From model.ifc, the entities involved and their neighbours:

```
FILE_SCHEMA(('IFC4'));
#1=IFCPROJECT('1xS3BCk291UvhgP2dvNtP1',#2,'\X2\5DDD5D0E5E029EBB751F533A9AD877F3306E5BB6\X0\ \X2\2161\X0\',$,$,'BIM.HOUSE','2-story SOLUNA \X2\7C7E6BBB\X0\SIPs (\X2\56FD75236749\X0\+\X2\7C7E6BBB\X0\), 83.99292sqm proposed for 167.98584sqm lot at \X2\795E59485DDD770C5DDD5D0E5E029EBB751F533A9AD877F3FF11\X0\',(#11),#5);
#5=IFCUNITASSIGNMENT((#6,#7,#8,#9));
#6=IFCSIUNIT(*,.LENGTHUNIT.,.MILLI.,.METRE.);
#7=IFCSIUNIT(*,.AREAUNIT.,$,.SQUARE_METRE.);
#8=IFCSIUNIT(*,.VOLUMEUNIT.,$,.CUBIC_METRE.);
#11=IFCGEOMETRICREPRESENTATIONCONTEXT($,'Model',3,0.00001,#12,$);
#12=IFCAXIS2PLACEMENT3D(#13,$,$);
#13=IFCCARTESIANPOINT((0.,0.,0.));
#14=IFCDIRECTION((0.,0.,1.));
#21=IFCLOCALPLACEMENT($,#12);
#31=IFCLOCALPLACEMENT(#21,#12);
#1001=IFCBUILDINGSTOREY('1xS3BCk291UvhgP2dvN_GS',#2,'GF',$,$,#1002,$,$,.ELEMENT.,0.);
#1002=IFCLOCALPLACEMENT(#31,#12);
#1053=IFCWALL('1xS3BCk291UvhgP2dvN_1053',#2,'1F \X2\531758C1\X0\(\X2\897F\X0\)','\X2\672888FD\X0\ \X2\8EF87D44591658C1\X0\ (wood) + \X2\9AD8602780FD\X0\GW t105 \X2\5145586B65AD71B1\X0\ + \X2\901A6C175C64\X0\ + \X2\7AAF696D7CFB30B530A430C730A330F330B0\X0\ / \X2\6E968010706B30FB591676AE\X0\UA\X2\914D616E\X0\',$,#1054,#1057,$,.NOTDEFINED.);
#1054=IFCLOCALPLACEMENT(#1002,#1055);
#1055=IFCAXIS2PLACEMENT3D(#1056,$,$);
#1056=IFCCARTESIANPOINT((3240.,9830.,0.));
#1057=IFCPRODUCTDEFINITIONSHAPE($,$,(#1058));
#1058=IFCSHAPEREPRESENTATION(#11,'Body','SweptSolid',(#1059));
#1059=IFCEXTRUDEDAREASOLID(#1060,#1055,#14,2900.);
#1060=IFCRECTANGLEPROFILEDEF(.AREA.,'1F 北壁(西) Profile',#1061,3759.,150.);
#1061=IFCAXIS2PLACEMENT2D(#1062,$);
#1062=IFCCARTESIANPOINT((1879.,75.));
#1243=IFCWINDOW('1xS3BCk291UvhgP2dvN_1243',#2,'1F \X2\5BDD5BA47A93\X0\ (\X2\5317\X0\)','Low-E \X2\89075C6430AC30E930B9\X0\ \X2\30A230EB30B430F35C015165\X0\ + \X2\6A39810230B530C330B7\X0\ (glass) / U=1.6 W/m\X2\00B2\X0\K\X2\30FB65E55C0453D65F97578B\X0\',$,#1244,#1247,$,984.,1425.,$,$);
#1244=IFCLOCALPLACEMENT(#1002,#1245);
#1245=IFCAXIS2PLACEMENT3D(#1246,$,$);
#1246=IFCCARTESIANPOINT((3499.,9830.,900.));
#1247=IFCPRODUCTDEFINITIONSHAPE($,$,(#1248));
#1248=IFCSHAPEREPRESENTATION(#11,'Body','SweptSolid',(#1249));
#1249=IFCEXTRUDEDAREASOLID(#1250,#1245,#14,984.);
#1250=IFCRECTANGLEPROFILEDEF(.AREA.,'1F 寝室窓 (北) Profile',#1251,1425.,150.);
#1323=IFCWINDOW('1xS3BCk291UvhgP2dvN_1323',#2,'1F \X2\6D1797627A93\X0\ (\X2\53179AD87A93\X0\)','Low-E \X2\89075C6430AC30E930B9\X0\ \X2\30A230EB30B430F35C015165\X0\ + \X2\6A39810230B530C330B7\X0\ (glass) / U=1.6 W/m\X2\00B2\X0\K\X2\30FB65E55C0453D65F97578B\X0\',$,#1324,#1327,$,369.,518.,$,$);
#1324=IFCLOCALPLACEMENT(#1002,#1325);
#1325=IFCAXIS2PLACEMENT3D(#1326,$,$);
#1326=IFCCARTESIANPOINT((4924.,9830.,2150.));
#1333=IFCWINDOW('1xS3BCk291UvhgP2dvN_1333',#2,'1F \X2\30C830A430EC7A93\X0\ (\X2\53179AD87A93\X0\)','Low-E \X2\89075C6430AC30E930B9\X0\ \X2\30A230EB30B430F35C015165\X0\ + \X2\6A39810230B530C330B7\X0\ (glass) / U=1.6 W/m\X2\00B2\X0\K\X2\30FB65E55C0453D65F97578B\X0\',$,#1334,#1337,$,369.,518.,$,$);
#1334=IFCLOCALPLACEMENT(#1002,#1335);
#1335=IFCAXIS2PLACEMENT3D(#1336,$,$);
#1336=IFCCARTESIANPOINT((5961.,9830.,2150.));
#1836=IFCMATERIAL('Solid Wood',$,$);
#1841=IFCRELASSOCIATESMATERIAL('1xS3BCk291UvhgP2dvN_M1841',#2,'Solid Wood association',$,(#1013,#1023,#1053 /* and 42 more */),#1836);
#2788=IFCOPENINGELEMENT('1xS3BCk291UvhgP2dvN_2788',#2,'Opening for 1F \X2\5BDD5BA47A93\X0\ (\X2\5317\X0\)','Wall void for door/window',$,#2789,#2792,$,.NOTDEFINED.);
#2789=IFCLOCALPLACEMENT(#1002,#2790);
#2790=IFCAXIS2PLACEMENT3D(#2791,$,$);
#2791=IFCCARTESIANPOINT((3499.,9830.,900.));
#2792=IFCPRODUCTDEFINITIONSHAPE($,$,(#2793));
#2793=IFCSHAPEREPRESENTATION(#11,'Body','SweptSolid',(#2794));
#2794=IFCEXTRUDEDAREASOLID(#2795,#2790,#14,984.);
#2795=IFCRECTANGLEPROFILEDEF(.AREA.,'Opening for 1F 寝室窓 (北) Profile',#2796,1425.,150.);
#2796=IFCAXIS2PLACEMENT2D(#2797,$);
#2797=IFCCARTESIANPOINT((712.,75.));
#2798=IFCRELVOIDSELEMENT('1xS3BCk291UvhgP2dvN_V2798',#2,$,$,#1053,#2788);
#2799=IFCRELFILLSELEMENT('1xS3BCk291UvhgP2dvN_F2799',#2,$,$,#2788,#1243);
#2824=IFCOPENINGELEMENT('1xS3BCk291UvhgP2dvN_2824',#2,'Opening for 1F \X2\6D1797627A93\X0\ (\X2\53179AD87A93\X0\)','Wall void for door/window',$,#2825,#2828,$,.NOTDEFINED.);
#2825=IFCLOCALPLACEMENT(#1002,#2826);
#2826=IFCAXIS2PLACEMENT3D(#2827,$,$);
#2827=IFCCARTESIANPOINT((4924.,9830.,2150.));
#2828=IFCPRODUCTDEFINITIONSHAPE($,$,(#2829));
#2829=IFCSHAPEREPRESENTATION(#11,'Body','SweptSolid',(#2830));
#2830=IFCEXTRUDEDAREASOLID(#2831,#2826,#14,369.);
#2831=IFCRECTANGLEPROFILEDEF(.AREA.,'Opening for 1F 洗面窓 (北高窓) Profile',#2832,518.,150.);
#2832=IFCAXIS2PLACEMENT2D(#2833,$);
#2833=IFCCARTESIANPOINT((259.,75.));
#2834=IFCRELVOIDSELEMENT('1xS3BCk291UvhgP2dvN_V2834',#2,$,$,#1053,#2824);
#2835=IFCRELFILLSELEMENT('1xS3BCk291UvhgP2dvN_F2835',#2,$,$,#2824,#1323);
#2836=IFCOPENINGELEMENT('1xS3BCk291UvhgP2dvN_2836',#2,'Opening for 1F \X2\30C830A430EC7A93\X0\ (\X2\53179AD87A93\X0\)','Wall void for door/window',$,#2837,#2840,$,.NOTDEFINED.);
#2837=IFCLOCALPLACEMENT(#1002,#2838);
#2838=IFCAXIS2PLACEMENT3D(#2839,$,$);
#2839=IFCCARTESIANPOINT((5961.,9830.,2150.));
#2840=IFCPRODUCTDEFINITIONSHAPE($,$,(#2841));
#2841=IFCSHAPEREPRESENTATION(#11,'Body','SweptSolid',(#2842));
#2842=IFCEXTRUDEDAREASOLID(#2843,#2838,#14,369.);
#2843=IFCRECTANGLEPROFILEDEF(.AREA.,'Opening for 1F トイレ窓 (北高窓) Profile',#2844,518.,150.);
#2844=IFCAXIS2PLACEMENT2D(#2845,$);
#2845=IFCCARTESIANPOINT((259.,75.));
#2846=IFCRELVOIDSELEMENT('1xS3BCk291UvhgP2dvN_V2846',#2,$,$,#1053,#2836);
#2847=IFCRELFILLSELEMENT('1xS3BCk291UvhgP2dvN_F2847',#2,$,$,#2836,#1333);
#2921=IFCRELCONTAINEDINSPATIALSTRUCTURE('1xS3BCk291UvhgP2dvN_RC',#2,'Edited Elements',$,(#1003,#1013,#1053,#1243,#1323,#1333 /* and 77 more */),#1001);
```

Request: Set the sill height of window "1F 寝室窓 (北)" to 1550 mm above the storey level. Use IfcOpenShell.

```python
import numpy as np
import ifcopenshell
import ifcopenshell.api.geometry
import ifcopenshell.geom
import ifcopenshell.util.element
import ifcopenshell.util.placement
import ifcopenshell.util.shape
import ifcopenshell.util.unit

model = ifcopenshell.open("model.ifc")
unit_scale = ifcopenshell.util.unit.calculate_unit_scale(model)

window = model.by_guid("1xS3BCk291UvhgP2dvN_1243")
opening = window.FillsVoids[0].RelatingOpeningElement
storey = ifcopenshell.util.element.get_container(window, ifc_class="IfcBuildingStorey")
level = ifcopenshell.util.placement.get_local_placement(storey.ObjectPlacement)[2, 3]

# The opening's origin need not be at the sill, so measure its lowest point.
shape = ifcopenshell.geom.create_shape(ifcopenshell.geom.settings(), opening)
bottom = ifcopenshell.util.shape.get_shape_bottom_elevation(shape, shape.geometry) / unit_scale
dz = level + 1550.0 - bottom

shift = np.array([0.0, 0.0, dz])
# The window is not placed relative to its opening, so move both.
for product in (opening, window):
    matrix = ifcopenshell.util.placement.get_local_placement(product.ObjectPlacement)
    matrix[:3, 3] += shift
    ifcopenshell.api.geometry.edit_object_placement(model, product=product, matrix=matrix, is_si=False)

print(f"moved by {dz * unit_scale:+.3f} m")

model.write("model-out.ifc")
```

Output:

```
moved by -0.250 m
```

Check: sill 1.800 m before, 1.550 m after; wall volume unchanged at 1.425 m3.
